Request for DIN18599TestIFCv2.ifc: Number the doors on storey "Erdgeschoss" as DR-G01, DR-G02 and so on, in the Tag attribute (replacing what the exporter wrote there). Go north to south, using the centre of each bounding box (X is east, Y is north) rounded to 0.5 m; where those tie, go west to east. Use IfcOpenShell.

First a look at what the model holds.

```python
import ifcopenshell
import ifcopenshell.util.element
import ifcopenshell.util.placement

model = ifcopenshell.open("DIN18599TestIFCv2.ifc")
print(model.schema)
storey = next(s for s in model.by_type("IfcBuildingStorey") if s.Name == "Erdgeschoss")
doors = [e for e in ifcopenshell.util.element.get_decomposition(storey) if e.is_a("IfcDoor")]
for e in sorted(doors, key=lambda e: e.id()):
    origin = ifcopenshell.util.placement.get_local_placement(e.ObjectPlacement)[:3, 3]
    print(e.id(), e.Tag, e.Name, origin.round(2) + 0.0, sep=" | ")
```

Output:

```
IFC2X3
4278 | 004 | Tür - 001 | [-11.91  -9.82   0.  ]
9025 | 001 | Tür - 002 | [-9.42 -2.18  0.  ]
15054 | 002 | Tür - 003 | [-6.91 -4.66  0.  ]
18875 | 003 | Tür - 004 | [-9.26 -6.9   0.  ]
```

```python
import ifcopenshell
import ifcopenshell.geom
import ifcopenshell.util.element
import ifcopenshell.util.shape

model = ifcopenshell.open("DIN18599TestIFCv2.ifc")
settings = ifcopenshell.geom.settings()
settings.set("use-world-coords", True)


def centre(element):
    shape = ifcopenshell.geom.create_shape(settings, element)
    return ifcopenshell.util.shape.get_bbox_centroid(shape.geometry)


storey = next(s for s in model.by_type("IfcBuildingStorey") if s.Name == "Erdgeschoss")
doors = [e for e in ifcopenshell.util.element.get_decomposition(storey) if e.is_a("IfcDoor")]

# Insertion points can sit at a corner or the storey origin, so sort by the geometry (in metres).
centres = {e: centre(e) for e in doors}
doors.sort(key=lambda e: (-round(centres[e][1] / 0.5), centres[e][0]))

for i, e in enumerate(doors, start=1):
    number = f"DR-G{i:02d}"
    e.Tag = number
    print(e.id(), number)

model.write("DIN18599TestIFCv2_updated.ifc")
```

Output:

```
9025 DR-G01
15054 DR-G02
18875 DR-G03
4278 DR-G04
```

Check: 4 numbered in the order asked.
